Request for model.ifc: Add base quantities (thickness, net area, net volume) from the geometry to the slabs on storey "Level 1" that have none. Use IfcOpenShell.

First a look at what the model holds.

```python
import ifcopenshell
import ifcopenshell.util.element
import ifcopenshell.util.unit

model = ifcopenshell.open("model.ifc")
print(model.schema)
for unit_type in ("LENGTHUNIT", "AREAUNIT", "VOLUMEUNIT"):
    print(unit_type, ifcopenshell.util.unit.calculate_unit_scale(model, unit_type))
storey = next(s for s in model.by_type("IfcBuildingStorey") if s.Name == "Level 1")
slabs = [e for e in ifcopenshell.util.element.get_decomposition(storey) if e.is_a("IfcSlab")]
for e in sorted(slabs, key=lambda e: e.id()):
    print(e.id(), e.is_a(), e.Name, list(ifcopenshell.util.element.get_psets(e, qtos_only=True)), sep=" | ")
```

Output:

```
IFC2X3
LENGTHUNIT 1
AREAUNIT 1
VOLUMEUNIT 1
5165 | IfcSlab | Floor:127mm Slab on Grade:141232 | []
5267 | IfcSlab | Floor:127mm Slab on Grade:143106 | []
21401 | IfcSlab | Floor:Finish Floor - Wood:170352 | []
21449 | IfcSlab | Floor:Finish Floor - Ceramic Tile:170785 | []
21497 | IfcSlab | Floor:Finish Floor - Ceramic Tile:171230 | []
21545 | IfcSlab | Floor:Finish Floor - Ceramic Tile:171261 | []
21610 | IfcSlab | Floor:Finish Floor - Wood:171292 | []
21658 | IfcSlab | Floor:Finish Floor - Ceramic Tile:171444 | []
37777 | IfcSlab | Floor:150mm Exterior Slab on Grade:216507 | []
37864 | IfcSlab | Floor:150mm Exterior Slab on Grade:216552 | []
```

```python
import ifcopenshell
import ifcopenshell.api.pset
import ifcopenshell.geom
import ifcopenshell.util.element
import ifcopenshell.util.shape
import ifcopenshell.util.unit

model = ifcopenshell.open("model.ifc")
unit_scale = ifcopenshell.util.unit.calculate_unit_scale(model)
area_scale = ifcopenshell.util.unit.calculate_unit_scale(model, "AREAUNIT")
volume_scale = ifcopenshell.util.unit.calculate_unit_scale(model, "VOLUMEUNIT")
settings = ifcopenshell.geom.settings()

storey = next(s for s in model.by_type("IfcBuildingStorey") if s.Name == "Level 1")
slabs = [e for e in ifcopenshell.util.element.get_decomposition(storey) if e.is_a("IfcSlab")]

for e in sorted(slabs, key=lambda e: e.id()):
    if ifcopenshell.util.element.get_psets(e, qtos_only=True, should_inherit=False):
        continue
    # Geometry comes back in metres, in the element's own axes.
    shape = ifcopenshell.geom.create_shape(settings, e)
    values = {
        "Width": ifcopenshell.util.shape.get_z(shape.geometry) / unit_scale,
        "NetArea": ifcopenshell.util.shape.get_footprint_area(shape.geometry) / area_scale,
        "NetVolume": ifcopenshell.util.shape.get_volume(shape.geometry) / volume_scale,
    }
    qto = ifcopenshell.api.pset.add_qto(model, product=e, name="BaseQuantities")
    ifcopenshell.api.pset.edit_qto(model, qto=qto, properties=values)
    print(e.id(), {k: round(v, 3) for k, v in values.items()})

model.write("model-out.ifc")
```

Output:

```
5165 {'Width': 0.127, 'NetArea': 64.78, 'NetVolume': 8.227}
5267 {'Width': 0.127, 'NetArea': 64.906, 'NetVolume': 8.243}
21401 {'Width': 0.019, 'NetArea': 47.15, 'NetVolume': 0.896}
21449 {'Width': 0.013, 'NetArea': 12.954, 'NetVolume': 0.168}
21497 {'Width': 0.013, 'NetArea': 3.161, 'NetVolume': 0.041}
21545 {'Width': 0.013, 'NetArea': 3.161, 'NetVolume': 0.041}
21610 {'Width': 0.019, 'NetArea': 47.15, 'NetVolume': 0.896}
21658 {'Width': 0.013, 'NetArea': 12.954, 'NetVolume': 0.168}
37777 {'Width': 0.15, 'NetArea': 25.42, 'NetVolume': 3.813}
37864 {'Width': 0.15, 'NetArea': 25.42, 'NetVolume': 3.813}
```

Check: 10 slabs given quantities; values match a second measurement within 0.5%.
